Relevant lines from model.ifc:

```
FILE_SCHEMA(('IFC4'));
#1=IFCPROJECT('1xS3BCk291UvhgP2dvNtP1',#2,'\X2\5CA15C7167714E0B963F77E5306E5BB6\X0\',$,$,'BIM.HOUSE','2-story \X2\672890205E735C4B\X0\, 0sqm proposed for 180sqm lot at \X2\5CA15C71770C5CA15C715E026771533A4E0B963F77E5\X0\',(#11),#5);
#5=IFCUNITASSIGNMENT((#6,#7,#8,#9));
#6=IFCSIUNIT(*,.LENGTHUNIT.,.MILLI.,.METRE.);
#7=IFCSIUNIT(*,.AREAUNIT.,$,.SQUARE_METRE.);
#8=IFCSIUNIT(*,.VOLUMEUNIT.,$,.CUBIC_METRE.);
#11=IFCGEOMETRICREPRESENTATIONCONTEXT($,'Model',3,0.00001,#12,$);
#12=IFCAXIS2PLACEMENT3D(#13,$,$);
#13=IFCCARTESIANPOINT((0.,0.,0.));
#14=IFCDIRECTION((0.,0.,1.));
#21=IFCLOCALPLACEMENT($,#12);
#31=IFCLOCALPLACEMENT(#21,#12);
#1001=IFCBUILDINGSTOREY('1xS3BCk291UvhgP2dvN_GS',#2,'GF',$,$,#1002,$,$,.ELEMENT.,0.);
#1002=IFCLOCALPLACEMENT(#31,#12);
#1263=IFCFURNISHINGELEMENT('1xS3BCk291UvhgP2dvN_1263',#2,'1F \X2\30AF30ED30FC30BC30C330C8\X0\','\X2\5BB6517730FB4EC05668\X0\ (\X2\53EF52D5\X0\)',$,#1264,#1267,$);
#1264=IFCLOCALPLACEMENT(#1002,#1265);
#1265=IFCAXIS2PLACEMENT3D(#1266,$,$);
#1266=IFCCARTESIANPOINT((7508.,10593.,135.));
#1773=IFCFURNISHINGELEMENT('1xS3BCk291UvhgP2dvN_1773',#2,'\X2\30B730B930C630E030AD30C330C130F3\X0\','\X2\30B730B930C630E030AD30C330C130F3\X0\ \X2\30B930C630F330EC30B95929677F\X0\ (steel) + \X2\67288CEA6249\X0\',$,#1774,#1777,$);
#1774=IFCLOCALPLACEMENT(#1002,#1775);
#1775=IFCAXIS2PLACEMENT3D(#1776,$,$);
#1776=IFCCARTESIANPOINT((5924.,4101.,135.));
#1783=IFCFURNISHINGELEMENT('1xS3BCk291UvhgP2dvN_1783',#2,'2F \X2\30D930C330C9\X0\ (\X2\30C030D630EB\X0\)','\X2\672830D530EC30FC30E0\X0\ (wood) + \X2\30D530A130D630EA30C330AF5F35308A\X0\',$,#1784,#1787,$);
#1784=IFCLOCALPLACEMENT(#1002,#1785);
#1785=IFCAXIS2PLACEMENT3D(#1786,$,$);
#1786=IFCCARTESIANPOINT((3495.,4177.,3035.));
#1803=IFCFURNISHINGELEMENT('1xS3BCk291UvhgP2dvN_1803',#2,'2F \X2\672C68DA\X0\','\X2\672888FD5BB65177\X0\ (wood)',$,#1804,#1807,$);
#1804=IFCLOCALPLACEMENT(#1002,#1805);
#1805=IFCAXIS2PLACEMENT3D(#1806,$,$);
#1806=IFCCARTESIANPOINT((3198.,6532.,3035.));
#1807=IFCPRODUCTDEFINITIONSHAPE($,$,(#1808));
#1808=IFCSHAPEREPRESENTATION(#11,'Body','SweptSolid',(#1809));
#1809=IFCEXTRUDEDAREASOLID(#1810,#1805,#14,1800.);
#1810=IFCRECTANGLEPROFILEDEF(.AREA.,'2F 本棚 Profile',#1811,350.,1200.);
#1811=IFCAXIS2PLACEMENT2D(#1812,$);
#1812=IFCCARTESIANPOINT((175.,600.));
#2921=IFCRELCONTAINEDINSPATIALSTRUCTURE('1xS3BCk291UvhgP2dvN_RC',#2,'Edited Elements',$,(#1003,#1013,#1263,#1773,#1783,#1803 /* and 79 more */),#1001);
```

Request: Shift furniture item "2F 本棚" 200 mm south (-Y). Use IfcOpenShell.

```python
import ifcopenshell
import ifcopenshell.api.geometry
import ifcopenshell.util.placement
import ifcopenshell.util.unit

model = ifcopenshell.open("model.ifc")
unit_scale = ifcopenshell.util.unit.calculate_unit_scale(model)

item = model.by_guid("1xS3BCk291UvhgP2dvN_1803")
matrix = ifcopenshell.util.placement.get_local_placement(item.ObjectPlacement)
matrix[1, 3] -= 0.2 / unit_scale
ifcopenshell.api.geometry.edit_object_placement(model, product=item, matrix=matrix, is_si=False)

print(ifcopenshell.util.placement.get_local_placement(item.ObjectPlacement).round(3) + 0.0)

model.write("model_v2.ifc")
```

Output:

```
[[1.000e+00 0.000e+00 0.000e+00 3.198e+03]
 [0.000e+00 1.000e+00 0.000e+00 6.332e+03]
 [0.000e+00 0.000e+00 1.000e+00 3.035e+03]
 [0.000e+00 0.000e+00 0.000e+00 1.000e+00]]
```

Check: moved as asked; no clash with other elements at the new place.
